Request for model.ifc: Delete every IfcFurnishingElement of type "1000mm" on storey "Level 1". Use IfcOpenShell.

First a look at what the model holds.

```python
import ifcopenshell
import ifcopenshell.util.element

model = ifcopenshell.open("model.ifc")
print(model.schema)
storey = next(s for s in model.by_type("IfcBuildingStorey") if s.Name == "Level 1")
furniture = [e for e in ifcopenshell.util.element.get_decomposition(storey) if e.is_a("IfcFurnishingElement")]
seen = {}
for e in furniture:
    element_type = ifcopenshell.util.element.get_type(e)
    name = element_type.Name if element_type not in (None, e) else None
    seen[name] = seen.get(name, 0) + 1
for name, count in sorted(seen.items(), key=str):
    print(count, "x", name)
```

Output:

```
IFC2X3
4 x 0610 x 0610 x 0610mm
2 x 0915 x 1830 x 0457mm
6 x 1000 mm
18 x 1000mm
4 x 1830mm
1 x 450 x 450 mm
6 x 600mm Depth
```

```python
import ifcopenshell
import ifcopenshell.api.root
import ifcopenshell.util.element

model = ifcopenshell.open("model.ifc")

storey = next(s for s in model.by_type("IfcBuildingStorey") if s.Name == "Level 1")
furniture = [e for e in ifcopenshell.util.element.get_decomposition(storey) if e.is_a("IfcFurnishingElement")]
targets = [e for e in furniture if (t := ifcopenshell.util.element.get_type(e)) not in (None, e) and t.Name == "1000mm"]

for e in targets:
    ifcopenshell.api.root.remove_product(model, product=e)
print(len(targets), "removed")

model.write("model_updated.ifc")
```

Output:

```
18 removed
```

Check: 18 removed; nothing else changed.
